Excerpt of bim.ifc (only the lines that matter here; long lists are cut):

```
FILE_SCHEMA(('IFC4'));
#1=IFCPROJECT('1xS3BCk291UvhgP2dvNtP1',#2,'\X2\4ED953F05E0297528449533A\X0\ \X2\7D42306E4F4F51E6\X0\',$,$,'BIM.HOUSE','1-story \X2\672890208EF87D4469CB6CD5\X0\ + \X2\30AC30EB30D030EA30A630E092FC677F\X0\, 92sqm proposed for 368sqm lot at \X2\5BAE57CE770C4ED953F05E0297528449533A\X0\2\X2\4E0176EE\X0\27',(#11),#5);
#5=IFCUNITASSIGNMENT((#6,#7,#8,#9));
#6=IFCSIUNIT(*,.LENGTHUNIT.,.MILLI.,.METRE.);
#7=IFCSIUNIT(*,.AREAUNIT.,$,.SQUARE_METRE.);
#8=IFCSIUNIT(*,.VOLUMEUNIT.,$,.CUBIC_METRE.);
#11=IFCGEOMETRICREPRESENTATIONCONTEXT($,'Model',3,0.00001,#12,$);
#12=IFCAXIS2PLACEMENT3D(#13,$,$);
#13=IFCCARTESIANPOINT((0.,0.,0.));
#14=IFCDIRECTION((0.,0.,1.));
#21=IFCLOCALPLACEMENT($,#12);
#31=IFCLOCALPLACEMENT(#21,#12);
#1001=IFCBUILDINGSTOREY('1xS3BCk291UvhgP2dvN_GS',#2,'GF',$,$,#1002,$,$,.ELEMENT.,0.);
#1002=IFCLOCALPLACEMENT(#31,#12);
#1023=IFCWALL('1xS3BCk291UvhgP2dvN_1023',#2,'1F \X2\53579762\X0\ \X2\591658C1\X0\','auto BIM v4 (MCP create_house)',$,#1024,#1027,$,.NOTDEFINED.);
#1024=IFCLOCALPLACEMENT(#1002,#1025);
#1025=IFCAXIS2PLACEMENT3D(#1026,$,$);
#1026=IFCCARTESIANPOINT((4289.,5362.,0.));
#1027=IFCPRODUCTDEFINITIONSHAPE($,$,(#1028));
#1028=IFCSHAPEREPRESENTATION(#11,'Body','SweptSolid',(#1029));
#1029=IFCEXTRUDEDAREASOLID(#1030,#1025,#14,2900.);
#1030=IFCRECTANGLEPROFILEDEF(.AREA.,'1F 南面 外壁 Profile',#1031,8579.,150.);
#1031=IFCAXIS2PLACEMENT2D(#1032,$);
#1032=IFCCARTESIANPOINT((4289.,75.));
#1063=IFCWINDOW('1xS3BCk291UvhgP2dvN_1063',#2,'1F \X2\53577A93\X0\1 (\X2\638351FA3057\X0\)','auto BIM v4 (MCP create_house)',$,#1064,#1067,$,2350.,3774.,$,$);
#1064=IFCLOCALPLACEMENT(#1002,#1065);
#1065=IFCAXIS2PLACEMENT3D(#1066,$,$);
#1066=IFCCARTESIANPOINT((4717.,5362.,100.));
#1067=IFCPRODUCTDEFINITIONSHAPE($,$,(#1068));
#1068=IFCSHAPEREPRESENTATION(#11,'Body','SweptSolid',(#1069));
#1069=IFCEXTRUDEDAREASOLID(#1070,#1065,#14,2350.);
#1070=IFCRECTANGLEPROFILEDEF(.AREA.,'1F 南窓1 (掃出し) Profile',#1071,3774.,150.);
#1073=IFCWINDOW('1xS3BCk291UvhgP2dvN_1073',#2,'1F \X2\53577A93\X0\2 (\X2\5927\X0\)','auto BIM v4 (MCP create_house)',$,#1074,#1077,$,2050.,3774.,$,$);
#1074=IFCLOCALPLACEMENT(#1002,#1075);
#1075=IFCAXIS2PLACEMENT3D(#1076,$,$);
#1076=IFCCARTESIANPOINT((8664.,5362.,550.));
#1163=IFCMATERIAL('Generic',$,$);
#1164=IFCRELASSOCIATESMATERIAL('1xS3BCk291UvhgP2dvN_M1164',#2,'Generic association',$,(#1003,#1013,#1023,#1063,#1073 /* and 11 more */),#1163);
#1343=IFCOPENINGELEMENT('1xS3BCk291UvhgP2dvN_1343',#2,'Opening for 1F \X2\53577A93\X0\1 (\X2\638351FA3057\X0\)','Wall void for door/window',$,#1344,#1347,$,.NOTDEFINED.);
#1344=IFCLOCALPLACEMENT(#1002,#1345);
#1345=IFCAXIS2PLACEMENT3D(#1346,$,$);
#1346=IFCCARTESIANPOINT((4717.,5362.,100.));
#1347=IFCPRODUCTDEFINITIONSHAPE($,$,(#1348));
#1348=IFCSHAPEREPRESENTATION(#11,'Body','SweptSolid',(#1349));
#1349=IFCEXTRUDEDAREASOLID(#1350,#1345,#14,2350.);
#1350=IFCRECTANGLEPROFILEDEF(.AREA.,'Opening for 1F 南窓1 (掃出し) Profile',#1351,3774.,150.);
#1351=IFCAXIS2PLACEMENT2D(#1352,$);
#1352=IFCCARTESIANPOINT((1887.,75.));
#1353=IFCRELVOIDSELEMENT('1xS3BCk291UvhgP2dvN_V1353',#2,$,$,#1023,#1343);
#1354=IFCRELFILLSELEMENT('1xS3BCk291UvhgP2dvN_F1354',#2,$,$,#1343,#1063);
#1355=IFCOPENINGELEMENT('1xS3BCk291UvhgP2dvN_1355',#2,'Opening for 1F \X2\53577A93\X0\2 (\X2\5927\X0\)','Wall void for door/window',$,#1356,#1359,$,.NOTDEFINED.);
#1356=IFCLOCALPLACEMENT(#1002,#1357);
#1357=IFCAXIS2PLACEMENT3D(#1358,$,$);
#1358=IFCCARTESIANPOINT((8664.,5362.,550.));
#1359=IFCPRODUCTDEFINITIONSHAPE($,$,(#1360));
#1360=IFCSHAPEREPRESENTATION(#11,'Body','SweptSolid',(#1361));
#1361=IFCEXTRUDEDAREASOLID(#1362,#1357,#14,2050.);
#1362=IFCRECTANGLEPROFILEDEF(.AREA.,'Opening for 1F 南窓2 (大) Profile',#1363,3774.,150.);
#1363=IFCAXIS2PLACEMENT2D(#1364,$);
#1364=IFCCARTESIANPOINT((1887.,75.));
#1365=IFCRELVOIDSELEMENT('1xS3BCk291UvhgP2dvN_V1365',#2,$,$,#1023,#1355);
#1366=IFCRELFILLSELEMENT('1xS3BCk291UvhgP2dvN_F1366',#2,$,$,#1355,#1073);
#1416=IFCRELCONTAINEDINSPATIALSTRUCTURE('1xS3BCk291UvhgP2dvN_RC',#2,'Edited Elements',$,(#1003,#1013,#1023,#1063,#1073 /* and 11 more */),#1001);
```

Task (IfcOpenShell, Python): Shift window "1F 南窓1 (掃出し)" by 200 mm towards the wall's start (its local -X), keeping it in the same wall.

```python
import ifcopenshell
import ifcopenshell.api.geometry
import ifcopenshell.util.placement
import ifcopenshell.util.unit

model = ifcopenshell.open("bim.ifc")
unit_scale = ifcopenshell.util.unit.calculate_unit_scale(model)

window = model.by_guid("1xS3BCk291UvhgP2dvN_1063")
opening = window.FillsVoids[0].RelatingOpeningElement
wall = opening.VoidsElements[0].RelatingBuildingElement

wall_matrix = ifcopenshell.util.placement.get_local_placement(wall.ObjectPlacement)
shift = wall_matrix[:3, 0] * -0.2 / unit_scale
before = ifcopenshell.util.placement.get_local_placement(window.ObjectPlacement)[:3, 3].copy()

# The window is not placed relative to its opening, so move both.
for product in (opening, window):
    matrix = ifcopenshell.util.placement.get_local_placement(product.ObjectPlacement)
    matrix[:3, 3] += shift
    ifcopenshell.api.geometry.edit_object_placement(model, product=product, matrix=matrix, is_si=False)

after = ifcopenshell.util.placement.get_local_placement(window.ObjectPlacement)[:3, 3]
print("window moved by", (after - before).round(3) + 0.0)

model.write("bim_v2.ifc")
```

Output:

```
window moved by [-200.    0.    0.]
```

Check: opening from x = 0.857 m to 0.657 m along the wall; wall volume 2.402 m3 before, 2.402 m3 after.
